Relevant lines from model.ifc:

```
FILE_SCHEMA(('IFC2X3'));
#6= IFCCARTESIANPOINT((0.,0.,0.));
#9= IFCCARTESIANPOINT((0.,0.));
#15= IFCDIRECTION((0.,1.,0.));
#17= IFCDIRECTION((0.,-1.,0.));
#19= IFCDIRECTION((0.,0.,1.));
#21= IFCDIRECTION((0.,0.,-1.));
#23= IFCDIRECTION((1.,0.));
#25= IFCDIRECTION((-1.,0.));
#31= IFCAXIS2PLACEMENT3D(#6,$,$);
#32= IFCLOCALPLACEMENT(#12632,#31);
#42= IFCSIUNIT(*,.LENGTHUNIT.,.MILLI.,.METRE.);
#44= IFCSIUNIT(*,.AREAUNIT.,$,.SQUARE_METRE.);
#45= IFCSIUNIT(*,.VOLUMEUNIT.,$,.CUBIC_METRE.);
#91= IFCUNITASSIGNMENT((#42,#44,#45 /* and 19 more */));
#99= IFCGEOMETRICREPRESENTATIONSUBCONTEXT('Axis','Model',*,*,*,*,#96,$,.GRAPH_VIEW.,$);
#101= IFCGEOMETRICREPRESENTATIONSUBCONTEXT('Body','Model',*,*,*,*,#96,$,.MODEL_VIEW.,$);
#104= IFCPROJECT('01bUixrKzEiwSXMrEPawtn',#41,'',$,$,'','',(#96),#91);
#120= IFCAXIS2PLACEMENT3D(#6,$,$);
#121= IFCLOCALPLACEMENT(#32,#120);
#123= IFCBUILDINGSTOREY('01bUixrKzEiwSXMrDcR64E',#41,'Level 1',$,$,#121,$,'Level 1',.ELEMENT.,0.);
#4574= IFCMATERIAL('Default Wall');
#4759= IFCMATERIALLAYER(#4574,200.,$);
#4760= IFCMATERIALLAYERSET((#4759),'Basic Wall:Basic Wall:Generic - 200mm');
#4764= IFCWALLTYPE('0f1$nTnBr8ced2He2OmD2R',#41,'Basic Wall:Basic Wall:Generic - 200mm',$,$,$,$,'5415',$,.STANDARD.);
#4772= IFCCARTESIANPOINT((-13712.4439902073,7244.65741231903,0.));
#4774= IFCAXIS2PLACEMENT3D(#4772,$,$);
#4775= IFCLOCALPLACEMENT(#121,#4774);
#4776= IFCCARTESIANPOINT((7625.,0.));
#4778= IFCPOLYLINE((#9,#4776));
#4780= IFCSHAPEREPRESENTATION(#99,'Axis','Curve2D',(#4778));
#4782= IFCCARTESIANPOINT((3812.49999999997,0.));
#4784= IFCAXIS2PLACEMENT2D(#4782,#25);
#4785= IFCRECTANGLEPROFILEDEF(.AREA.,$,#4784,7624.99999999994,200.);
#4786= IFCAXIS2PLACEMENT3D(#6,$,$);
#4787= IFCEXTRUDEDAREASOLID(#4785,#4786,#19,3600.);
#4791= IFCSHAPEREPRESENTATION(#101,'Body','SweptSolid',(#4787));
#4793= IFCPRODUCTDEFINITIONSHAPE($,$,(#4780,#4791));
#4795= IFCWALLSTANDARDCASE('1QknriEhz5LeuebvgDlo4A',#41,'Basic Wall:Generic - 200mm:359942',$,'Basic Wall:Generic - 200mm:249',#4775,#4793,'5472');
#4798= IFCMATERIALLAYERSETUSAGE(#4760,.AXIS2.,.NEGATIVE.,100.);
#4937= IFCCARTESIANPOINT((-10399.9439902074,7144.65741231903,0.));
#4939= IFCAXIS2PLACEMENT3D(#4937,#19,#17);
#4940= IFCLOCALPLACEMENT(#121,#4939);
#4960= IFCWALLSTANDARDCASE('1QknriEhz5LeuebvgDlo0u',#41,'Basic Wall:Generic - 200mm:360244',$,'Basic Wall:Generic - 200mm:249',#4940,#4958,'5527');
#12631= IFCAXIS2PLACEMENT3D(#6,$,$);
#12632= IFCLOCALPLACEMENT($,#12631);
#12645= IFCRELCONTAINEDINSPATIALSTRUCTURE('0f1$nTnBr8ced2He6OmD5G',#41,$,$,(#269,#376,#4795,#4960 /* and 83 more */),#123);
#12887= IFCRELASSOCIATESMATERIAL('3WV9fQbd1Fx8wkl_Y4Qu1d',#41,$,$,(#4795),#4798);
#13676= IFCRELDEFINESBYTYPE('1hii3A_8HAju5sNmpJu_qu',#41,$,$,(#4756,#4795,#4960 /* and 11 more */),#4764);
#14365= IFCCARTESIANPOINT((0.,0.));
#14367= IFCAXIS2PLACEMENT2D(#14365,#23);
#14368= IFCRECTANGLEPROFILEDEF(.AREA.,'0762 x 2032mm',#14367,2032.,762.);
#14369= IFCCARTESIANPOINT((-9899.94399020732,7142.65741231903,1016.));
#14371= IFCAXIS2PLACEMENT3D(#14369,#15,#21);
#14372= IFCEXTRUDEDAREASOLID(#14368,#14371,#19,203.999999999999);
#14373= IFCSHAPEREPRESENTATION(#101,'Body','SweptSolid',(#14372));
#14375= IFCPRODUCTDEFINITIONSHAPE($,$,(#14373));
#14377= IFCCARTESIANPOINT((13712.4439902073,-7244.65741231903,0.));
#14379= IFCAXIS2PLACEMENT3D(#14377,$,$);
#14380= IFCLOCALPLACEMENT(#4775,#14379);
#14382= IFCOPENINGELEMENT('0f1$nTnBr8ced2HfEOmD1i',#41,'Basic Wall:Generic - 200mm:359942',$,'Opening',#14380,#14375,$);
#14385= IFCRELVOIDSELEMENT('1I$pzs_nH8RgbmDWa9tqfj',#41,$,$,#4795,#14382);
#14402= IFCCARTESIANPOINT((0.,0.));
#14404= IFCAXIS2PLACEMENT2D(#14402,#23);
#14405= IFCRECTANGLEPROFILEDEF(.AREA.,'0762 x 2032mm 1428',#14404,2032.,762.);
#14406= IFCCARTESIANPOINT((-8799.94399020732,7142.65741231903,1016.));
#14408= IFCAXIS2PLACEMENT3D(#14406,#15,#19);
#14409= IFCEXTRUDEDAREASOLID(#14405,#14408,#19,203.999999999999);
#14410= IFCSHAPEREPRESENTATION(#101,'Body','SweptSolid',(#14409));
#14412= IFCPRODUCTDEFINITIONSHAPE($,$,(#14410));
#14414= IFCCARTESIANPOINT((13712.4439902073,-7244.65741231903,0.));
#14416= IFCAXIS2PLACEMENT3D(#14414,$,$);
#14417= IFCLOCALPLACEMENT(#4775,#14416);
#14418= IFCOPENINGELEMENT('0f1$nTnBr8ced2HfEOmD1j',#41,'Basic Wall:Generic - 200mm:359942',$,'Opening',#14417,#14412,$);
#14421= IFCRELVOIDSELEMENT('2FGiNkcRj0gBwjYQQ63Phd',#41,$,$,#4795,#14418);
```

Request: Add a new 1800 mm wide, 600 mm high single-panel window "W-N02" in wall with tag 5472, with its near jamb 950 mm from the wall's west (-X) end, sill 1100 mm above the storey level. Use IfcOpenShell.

```python
import numpy as np
import ifcopenshell
import ifcopenshell.api.feature
import ifcopenshell.api.geometry
import ifcopenshell.api.root
import ifcopenshell.api.spatial
import ifcopenshell.api.type
import ifcopenshell.geom
import ifcopenshell.util.element
import ifcopenshell.util.placement
import ifcopenshell.util.representation
import ifcopenshell.util.shape
import ifcopenshell.util.unit

model = ifcopenshell.open("model.ifc")
unit_scale = ifcopenshell.util.unit.calculate_unit_scale(model)
settings = ifcopenshell.geom.settings()


def volume(element):
    """Net volume in cubic metres, openings subtracted."""
    shape = ifcopenshell.geom.create_shape(settings, element)
    return ifcopenshell.util.shape.get_volume(shape.geometry)


wall = model.by_guid("1QknriEhz5LeuebvgDlo4A")
storey = ifcopenshell.util.element.get_container(wall, ifc_class="IfcBuildingStorey")
context = ifcopenshell.util.representation.get_context(model, "Model", "Body", "MODEL_VIEW")
before = volume(wall)

width, height, from_end, sill = 1.8, 0.6, 0.95, 1.1  # metres

# The wall runs along its own X axis, and the end named is its -X end.
wall_shape = ifcopenshell.geom.create_shape(settings, wall)
x, y, z = ifcopenshell.util.shape.get_vertices(wall_shape.geometry).T
start = x.min() + from_end
face, thickness = float(y.min()), float(y.max() - y.min())
wall_matrix = ifcopenshell.util.placement.get_local_placement(wall.ObjectPlacement)
level = ifcopenshell.util.placement.get_local_placement(storey.ObjectPlacement)[2, 3]


def in_wall(x, y):
    """Placement at x, y metres in the wall's axes, at sill height."""
    matrix = wall_matrix.copy()
    matrix[:, 3] = wall_matrix @ np.array([x / unit_scale, y / unit_scale, 0.0, 1.0])
    matrix[2, 3] = level + sill / unit_scale
    return matrix


# Opening: a box that overshoots both wall faces by 50 mm.
opening = ifcopenshell.api.root.create_entity(model, ifc_class="IfcOpeningElement")
box = ifcopenshell.api.geometry.add_wall_representation(
    model, context=context, length=width, height=height, thickness=thickness + 0.1
)
ifcopenshell.api.geometry.assign_representation(model, product=opening, representation=box)
ifcopenshell.api.geometry.edit_object_placement(model, product=opening, matrix=in_wall(start, face - 0.05), is_si=False)
ifcopenshell.api.feature.add_feature(model, feature=opening, element=wall)

window = ifcopenshell.api.root.create_entity(model, ifc_class="IfcWindow", name="W-N02")
window.OverallWidth, window.OverallHeight = width / unit_scale, height / unit_scale
body = ifcopenshell.api.geometry.add_window_representation(
    model,
    context=context,
    overall_width=window.OverallWidth,
    overall_height=window.OverallHeight,
    partition_type="SINGLE_PANEL",
)
ifcopenshell.api.geometry.assign_representation(model, product=window, representation=body)
ifcopenshell.api.spatial.assign_container(model, products=[window], relating_structure=storey)
fills = ifcopenshell.api.feature.add_filling(model, opening=opening, element=window)
fills.OwnerHistory = window.OwnerHistory  # required in IFC2X3

# IFC2X3 keeps the operation on the window style.
style = ifcopenshell.api.root.create_entity(model, ifc_class="IfcWindowStyle", name="W-N02")
style.OperationType, style.ConstructionType = "SINGLE_PANEL", "NOTDEFINED"
style.ParameterTakesPrecedence = style.Sizeable = False
ifcopenshell.api.type.assign_type(model, related_objects=[window], relating_type=style)

# Centre the window in the wall's thickness.
ifcopenshell.api.geometry.edit_object_placement(model, product=window, matrix=in_wall(start, face), is_si=False)
window_shape = ifcopenshell.geom.create_shape(settings, window)
depth = ifcopenshell.util.shape.get_vertices(window_shape.geometry)[:, 1]
offset = face + thickness / 2 - (depth.min() + depth.max()) / 2
ifcopenshell.api.geometry.edit_object_placement(model, product=window, matrix=in_wall(start, offset), is_si=False)

after = volume(wall)

print(f"wall volume {before:.3f} -> {after:.3f} m3")

model.write("model_rev.ifc")
```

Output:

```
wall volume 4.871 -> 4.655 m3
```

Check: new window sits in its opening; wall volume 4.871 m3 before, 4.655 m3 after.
